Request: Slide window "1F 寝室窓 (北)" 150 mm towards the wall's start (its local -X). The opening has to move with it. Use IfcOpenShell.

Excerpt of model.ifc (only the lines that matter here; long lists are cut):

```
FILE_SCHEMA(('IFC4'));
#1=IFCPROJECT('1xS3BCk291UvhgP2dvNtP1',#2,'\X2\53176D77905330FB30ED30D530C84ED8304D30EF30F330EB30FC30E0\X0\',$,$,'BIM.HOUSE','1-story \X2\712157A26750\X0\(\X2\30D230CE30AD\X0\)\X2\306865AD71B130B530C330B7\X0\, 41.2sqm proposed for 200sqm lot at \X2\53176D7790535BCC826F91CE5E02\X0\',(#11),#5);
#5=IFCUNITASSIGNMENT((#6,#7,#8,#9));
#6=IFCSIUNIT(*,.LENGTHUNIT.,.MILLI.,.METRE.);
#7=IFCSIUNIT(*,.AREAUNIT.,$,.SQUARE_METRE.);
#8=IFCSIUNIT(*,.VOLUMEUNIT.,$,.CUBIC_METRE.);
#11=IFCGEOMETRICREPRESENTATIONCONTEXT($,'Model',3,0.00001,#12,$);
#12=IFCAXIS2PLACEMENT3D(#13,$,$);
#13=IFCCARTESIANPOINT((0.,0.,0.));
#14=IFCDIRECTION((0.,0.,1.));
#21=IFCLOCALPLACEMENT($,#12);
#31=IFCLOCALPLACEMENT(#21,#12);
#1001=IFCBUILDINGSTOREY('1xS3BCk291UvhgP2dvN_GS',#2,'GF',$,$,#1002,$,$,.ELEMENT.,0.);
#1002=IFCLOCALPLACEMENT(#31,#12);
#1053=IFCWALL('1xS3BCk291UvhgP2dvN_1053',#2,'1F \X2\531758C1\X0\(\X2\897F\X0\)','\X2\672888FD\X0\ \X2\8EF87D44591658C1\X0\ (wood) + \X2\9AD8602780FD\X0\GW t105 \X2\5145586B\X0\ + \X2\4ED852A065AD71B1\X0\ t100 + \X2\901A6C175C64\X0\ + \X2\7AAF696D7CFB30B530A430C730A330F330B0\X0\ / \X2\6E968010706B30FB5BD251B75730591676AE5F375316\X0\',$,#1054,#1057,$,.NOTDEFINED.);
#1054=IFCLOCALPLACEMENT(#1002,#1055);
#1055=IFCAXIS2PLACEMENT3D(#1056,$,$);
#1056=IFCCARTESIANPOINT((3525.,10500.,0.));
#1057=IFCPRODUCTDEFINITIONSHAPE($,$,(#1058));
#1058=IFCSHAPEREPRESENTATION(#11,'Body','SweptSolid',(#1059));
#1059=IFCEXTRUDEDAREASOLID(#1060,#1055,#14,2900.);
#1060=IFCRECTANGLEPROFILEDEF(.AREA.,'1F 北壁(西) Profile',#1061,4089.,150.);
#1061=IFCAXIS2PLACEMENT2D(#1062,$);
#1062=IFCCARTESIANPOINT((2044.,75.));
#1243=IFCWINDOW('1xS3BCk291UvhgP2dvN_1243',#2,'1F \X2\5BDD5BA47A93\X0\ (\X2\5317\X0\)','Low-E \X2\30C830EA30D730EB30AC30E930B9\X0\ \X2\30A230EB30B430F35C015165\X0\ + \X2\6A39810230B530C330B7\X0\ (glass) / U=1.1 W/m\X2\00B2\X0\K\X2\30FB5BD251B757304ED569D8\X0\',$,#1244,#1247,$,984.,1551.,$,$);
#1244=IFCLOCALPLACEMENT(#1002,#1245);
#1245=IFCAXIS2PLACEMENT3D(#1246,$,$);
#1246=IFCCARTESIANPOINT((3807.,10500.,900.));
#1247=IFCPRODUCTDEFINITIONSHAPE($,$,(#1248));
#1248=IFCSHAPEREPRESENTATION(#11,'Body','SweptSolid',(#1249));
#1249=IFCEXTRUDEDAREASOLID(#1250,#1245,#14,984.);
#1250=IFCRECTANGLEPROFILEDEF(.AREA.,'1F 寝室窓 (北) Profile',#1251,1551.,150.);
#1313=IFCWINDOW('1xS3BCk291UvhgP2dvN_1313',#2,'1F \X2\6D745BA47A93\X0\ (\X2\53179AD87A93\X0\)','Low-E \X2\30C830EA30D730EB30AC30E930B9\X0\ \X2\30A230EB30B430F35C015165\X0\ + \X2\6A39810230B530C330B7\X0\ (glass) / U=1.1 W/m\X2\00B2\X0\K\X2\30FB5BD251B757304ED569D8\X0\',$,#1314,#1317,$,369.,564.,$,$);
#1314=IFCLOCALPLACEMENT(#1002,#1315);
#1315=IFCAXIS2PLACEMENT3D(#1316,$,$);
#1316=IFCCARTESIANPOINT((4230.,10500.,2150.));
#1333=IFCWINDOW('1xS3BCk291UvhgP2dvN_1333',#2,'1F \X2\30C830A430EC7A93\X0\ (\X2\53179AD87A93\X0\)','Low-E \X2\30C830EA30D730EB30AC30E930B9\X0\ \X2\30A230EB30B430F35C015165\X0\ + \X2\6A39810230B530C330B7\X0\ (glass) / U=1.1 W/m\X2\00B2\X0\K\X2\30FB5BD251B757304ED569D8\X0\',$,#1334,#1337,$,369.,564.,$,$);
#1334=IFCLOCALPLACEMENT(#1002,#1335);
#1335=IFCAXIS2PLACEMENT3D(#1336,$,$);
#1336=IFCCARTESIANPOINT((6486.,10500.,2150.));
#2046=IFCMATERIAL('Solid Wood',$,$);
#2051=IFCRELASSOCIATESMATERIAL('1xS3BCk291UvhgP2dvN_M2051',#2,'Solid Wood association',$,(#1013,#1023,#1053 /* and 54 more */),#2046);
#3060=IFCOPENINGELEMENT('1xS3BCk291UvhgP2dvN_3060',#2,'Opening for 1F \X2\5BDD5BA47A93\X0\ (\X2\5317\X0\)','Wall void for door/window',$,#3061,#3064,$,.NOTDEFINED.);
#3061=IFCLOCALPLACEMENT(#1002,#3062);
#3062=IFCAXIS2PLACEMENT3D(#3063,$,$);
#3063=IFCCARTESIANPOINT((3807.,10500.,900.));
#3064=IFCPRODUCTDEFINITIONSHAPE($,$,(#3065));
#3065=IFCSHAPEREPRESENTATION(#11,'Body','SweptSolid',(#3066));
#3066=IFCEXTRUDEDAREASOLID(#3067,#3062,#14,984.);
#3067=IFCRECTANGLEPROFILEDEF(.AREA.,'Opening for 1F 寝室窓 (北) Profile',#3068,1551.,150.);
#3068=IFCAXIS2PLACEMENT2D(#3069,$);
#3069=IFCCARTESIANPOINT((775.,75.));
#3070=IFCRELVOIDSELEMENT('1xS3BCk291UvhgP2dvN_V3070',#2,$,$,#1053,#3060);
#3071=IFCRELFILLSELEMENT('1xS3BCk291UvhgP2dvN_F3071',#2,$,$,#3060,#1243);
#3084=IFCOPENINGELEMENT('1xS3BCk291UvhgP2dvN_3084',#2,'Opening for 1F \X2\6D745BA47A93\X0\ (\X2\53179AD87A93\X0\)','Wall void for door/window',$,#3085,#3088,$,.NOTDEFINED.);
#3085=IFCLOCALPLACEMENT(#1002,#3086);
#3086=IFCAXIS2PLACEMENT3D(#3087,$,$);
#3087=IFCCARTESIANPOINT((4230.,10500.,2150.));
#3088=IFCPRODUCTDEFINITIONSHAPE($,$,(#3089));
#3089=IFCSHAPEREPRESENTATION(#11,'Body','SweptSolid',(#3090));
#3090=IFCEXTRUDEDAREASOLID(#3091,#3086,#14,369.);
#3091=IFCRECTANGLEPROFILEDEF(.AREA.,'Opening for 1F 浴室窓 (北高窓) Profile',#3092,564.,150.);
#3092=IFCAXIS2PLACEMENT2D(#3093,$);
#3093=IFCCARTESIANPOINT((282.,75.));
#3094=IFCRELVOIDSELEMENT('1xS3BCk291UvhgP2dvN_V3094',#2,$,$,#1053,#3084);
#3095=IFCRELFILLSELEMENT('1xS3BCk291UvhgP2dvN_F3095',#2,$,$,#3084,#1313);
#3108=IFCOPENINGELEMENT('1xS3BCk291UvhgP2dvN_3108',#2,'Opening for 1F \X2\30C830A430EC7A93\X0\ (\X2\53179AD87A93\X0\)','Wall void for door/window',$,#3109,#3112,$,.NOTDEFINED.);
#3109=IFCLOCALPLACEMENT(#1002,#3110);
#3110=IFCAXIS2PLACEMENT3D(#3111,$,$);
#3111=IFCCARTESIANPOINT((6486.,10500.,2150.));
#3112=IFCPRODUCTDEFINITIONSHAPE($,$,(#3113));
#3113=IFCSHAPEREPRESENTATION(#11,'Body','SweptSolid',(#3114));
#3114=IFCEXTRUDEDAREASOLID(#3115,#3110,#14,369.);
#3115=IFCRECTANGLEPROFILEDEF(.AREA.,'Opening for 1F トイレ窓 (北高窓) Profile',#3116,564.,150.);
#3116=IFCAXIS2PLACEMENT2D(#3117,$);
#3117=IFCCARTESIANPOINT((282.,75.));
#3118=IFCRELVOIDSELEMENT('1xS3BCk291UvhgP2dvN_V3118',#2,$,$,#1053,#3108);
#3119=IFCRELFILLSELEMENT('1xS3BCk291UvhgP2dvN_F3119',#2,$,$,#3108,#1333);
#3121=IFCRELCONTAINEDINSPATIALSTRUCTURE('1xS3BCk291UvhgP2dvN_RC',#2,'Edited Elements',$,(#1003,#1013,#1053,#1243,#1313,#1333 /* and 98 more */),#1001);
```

```python
import ifcopenshell
import ifcopenshell.api.geometry
import ifcopenshell.util.placement
import ifcopenshell.util.unit

model = ifcopenshell.open("model.ifc")
unit_scale = ifcopenshell.util.unit.calculate_unit_scale(model)

window = model.by_guid("1xS3BCk291UvhgP2dvN_1243")
opening = window.FillsVoids[0].RelatingOpeningElement
wall = opening.VoidsElements[0].RelatingBuildingElement

wall_matrix = ifcopenshell.util.placement.get_local_placement(wall.ObjectPlacement)
shift = wall_matrix[:3, 0] * -0.15 / unit_scale
before = ifcopenshell.util.placement.get_local_placement(window.ObjectPlacement)[:3, 3].copy()

# The window is not placed relative to its opening, so move both.
for product in (opening, window):
    matrix = ifcopenshell.util.placement.get_local_placement(product.ObjectPlacement)
    matrix[:3, 3] += shift
    ifcopenshell.api.geometry.edit_object_placement(model, product=product, matrix=matrix, is_si=False)

after = ifcopenshell.util.placement.get_local_placement(window.ObjectPlacement)[:3, 3]
print("window moved by", (after - before).round(3) + 0.0)

model.write("model_rev.ifc")
```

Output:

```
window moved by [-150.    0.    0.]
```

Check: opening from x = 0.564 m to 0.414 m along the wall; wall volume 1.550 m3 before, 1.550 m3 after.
